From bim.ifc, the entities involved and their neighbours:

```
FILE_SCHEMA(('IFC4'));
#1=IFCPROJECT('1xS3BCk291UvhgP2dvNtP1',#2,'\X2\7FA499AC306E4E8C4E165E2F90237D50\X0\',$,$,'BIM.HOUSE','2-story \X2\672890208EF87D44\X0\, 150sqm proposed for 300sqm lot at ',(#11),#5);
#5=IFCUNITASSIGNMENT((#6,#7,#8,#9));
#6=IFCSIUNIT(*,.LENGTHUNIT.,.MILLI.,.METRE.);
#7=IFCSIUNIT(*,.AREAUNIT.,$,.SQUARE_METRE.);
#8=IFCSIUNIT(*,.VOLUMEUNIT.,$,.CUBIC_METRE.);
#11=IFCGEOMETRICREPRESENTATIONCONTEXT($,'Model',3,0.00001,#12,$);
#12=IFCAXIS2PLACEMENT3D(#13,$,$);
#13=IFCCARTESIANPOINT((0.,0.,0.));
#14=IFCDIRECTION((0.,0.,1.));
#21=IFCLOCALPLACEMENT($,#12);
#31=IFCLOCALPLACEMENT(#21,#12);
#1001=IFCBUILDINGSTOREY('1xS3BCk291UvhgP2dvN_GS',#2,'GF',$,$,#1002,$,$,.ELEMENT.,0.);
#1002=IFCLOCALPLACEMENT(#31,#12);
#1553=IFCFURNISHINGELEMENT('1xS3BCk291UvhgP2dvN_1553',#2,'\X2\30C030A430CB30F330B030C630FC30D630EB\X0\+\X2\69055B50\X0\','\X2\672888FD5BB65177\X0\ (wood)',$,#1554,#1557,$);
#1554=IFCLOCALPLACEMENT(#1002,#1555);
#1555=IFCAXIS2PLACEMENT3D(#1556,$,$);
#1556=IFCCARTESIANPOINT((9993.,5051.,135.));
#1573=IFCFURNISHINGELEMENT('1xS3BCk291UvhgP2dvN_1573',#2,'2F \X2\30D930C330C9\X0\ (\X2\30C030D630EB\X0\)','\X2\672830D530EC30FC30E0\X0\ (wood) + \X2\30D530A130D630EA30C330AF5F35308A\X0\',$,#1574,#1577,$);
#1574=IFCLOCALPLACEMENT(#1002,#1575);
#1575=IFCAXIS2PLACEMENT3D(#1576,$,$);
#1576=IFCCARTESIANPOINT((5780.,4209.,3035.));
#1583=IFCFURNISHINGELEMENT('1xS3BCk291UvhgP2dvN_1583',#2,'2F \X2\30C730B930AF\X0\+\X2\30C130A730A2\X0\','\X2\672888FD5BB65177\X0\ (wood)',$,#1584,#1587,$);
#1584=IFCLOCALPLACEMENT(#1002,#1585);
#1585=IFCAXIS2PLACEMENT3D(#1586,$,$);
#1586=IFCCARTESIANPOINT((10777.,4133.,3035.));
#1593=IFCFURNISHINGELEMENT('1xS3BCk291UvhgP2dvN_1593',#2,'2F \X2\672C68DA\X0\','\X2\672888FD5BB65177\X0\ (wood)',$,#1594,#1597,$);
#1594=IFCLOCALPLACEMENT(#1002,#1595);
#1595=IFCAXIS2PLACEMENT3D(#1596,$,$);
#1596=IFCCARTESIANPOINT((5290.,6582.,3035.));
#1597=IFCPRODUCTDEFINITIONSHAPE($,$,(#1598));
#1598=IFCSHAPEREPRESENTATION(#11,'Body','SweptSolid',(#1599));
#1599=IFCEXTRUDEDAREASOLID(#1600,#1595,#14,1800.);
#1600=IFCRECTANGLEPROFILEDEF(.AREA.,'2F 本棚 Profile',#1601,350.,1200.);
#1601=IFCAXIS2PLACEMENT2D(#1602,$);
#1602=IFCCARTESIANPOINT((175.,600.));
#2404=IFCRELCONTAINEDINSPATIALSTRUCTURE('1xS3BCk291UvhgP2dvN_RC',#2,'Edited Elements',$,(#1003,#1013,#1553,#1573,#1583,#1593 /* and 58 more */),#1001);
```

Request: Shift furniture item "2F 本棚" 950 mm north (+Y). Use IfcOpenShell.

```python
import ifcopenshell
import ifcopenshell.api.geometry
import ifcopenshell.util.placement

model = ifcopenshell.open("bim.ifc")

item = model.by_id(1593)
matrix = ifcopenshell.util.placement.get_local_placement(item.ObjectPlacement)
matrix[1, 3] += 950.0
ifcopenshell.api.geometry.edit_object_placement(model, product=item, matrix=matrix, is_si=False)

print(ifcopenshell.util.placement.get_local_placement(item.ObjectPlacement).round(3) + 0.0)

model.write("bim_v2.ifc")
```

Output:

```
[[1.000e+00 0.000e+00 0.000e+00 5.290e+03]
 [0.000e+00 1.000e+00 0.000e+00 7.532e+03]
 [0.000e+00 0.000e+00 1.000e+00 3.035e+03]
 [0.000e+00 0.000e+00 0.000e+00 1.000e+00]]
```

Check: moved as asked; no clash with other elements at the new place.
